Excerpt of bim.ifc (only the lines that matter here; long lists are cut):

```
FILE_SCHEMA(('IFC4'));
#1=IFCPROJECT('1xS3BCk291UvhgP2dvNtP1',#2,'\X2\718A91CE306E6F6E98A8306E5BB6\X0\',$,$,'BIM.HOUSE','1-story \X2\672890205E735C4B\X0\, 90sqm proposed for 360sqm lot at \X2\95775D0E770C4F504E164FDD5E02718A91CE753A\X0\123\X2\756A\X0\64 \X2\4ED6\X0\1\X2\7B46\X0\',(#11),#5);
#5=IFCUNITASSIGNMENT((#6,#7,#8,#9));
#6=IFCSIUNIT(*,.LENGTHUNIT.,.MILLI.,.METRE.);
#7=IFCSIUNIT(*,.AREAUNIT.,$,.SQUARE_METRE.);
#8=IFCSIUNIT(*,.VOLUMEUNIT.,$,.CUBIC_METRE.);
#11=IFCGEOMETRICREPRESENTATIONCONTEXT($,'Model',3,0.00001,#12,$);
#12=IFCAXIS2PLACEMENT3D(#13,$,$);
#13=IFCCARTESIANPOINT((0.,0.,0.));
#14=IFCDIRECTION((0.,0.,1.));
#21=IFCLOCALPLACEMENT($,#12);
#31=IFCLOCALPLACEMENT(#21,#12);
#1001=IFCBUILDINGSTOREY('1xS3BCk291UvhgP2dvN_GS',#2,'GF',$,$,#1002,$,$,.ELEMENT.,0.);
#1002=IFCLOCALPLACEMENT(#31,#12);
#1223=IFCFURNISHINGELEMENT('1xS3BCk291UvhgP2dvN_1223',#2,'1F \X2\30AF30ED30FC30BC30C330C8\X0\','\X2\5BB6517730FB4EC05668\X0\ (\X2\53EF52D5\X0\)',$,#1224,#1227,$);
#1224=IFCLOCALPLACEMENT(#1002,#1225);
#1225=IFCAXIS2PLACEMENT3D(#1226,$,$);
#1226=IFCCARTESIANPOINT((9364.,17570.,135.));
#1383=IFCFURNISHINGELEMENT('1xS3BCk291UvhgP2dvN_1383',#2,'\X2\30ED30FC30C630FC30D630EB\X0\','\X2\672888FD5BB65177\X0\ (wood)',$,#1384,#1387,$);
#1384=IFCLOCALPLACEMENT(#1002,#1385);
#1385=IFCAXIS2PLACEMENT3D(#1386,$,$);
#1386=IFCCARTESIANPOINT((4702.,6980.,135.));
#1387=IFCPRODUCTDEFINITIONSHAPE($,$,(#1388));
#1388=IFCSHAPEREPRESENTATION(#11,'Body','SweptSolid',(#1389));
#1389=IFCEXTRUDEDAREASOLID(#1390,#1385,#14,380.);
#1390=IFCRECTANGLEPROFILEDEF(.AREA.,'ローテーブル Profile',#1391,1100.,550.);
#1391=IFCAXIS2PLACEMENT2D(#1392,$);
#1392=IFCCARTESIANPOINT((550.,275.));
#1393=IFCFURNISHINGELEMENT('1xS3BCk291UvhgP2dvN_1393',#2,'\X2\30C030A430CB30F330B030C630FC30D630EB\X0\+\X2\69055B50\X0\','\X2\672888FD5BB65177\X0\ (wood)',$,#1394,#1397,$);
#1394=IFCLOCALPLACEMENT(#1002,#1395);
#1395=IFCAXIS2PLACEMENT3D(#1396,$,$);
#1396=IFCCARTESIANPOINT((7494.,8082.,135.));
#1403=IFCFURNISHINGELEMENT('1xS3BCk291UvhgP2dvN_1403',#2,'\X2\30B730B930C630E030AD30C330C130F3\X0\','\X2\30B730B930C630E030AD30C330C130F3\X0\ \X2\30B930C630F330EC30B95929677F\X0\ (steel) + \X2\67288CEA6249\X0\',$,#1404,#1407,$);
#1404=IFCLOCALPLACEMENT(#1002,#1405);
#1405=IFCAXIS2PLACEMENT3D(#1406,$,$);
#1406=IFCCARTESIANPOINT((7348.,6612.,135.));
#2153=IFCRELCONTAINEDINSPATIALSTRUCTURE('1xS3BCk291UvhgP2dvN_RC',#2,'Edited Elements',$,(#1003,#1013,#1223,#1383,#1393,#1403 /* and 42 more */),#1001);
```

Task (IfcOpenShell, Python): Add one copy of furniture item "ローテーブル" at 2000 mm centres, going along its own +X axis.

```python
import ifcopenshell
import ifcopenshell.api.geometry
import ifcopenshell.api.root
import ifcopenshell.util.element
import ifcopenshell.util.placement

model = ifcopenshell.open("bim.ifc")


def reuse_history(source, copy):
    """copy_class also copies each property set's owner history, people and application; keep the originals."""
    for rel in copy.IsDefinedBy:
        if rel.is_a("IfcRelDefinesByProperties") and (history := rel.RelatingPropertyDefinition.OwnerHistory):
            rel.RelatingPropertyDefinition.OwnerHistory = source.OwnerHistory
            ifcopenshell.util.element.remove_deep2(model, history)


source = model.by_guid("1xS3BCk291UvhgP2dvN_1383")
base = ifcopenshell.util.placement.get_local_placement(source.ObjectPlacement)
step = base[:3, 0] * 2000.0

for i in range(1, 2):
    copy = ifcopenshell.api.root.copy_class(model, product=source)
    copy.Representation = ifcopenshell.util.element.copy_deep(
        model, source.Representation, exclude=["IfcGeometricRepresentationContext", "IfcRepresentationMap"]
    )
    reuse_history(source, copy)
    matrix = base.copy()
    matrix[:3, 3] += i * step
    print("added at", matrix[:3, 3].round(3) + 0.0)
    ifcopenshell.api.geometry.edit_object_placement(model, product=copy, matrix=matrix, is_si=False)

model.write("bim_edited.ifc")
```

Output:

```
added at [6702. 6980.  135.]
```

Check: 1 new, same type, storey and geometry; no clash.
